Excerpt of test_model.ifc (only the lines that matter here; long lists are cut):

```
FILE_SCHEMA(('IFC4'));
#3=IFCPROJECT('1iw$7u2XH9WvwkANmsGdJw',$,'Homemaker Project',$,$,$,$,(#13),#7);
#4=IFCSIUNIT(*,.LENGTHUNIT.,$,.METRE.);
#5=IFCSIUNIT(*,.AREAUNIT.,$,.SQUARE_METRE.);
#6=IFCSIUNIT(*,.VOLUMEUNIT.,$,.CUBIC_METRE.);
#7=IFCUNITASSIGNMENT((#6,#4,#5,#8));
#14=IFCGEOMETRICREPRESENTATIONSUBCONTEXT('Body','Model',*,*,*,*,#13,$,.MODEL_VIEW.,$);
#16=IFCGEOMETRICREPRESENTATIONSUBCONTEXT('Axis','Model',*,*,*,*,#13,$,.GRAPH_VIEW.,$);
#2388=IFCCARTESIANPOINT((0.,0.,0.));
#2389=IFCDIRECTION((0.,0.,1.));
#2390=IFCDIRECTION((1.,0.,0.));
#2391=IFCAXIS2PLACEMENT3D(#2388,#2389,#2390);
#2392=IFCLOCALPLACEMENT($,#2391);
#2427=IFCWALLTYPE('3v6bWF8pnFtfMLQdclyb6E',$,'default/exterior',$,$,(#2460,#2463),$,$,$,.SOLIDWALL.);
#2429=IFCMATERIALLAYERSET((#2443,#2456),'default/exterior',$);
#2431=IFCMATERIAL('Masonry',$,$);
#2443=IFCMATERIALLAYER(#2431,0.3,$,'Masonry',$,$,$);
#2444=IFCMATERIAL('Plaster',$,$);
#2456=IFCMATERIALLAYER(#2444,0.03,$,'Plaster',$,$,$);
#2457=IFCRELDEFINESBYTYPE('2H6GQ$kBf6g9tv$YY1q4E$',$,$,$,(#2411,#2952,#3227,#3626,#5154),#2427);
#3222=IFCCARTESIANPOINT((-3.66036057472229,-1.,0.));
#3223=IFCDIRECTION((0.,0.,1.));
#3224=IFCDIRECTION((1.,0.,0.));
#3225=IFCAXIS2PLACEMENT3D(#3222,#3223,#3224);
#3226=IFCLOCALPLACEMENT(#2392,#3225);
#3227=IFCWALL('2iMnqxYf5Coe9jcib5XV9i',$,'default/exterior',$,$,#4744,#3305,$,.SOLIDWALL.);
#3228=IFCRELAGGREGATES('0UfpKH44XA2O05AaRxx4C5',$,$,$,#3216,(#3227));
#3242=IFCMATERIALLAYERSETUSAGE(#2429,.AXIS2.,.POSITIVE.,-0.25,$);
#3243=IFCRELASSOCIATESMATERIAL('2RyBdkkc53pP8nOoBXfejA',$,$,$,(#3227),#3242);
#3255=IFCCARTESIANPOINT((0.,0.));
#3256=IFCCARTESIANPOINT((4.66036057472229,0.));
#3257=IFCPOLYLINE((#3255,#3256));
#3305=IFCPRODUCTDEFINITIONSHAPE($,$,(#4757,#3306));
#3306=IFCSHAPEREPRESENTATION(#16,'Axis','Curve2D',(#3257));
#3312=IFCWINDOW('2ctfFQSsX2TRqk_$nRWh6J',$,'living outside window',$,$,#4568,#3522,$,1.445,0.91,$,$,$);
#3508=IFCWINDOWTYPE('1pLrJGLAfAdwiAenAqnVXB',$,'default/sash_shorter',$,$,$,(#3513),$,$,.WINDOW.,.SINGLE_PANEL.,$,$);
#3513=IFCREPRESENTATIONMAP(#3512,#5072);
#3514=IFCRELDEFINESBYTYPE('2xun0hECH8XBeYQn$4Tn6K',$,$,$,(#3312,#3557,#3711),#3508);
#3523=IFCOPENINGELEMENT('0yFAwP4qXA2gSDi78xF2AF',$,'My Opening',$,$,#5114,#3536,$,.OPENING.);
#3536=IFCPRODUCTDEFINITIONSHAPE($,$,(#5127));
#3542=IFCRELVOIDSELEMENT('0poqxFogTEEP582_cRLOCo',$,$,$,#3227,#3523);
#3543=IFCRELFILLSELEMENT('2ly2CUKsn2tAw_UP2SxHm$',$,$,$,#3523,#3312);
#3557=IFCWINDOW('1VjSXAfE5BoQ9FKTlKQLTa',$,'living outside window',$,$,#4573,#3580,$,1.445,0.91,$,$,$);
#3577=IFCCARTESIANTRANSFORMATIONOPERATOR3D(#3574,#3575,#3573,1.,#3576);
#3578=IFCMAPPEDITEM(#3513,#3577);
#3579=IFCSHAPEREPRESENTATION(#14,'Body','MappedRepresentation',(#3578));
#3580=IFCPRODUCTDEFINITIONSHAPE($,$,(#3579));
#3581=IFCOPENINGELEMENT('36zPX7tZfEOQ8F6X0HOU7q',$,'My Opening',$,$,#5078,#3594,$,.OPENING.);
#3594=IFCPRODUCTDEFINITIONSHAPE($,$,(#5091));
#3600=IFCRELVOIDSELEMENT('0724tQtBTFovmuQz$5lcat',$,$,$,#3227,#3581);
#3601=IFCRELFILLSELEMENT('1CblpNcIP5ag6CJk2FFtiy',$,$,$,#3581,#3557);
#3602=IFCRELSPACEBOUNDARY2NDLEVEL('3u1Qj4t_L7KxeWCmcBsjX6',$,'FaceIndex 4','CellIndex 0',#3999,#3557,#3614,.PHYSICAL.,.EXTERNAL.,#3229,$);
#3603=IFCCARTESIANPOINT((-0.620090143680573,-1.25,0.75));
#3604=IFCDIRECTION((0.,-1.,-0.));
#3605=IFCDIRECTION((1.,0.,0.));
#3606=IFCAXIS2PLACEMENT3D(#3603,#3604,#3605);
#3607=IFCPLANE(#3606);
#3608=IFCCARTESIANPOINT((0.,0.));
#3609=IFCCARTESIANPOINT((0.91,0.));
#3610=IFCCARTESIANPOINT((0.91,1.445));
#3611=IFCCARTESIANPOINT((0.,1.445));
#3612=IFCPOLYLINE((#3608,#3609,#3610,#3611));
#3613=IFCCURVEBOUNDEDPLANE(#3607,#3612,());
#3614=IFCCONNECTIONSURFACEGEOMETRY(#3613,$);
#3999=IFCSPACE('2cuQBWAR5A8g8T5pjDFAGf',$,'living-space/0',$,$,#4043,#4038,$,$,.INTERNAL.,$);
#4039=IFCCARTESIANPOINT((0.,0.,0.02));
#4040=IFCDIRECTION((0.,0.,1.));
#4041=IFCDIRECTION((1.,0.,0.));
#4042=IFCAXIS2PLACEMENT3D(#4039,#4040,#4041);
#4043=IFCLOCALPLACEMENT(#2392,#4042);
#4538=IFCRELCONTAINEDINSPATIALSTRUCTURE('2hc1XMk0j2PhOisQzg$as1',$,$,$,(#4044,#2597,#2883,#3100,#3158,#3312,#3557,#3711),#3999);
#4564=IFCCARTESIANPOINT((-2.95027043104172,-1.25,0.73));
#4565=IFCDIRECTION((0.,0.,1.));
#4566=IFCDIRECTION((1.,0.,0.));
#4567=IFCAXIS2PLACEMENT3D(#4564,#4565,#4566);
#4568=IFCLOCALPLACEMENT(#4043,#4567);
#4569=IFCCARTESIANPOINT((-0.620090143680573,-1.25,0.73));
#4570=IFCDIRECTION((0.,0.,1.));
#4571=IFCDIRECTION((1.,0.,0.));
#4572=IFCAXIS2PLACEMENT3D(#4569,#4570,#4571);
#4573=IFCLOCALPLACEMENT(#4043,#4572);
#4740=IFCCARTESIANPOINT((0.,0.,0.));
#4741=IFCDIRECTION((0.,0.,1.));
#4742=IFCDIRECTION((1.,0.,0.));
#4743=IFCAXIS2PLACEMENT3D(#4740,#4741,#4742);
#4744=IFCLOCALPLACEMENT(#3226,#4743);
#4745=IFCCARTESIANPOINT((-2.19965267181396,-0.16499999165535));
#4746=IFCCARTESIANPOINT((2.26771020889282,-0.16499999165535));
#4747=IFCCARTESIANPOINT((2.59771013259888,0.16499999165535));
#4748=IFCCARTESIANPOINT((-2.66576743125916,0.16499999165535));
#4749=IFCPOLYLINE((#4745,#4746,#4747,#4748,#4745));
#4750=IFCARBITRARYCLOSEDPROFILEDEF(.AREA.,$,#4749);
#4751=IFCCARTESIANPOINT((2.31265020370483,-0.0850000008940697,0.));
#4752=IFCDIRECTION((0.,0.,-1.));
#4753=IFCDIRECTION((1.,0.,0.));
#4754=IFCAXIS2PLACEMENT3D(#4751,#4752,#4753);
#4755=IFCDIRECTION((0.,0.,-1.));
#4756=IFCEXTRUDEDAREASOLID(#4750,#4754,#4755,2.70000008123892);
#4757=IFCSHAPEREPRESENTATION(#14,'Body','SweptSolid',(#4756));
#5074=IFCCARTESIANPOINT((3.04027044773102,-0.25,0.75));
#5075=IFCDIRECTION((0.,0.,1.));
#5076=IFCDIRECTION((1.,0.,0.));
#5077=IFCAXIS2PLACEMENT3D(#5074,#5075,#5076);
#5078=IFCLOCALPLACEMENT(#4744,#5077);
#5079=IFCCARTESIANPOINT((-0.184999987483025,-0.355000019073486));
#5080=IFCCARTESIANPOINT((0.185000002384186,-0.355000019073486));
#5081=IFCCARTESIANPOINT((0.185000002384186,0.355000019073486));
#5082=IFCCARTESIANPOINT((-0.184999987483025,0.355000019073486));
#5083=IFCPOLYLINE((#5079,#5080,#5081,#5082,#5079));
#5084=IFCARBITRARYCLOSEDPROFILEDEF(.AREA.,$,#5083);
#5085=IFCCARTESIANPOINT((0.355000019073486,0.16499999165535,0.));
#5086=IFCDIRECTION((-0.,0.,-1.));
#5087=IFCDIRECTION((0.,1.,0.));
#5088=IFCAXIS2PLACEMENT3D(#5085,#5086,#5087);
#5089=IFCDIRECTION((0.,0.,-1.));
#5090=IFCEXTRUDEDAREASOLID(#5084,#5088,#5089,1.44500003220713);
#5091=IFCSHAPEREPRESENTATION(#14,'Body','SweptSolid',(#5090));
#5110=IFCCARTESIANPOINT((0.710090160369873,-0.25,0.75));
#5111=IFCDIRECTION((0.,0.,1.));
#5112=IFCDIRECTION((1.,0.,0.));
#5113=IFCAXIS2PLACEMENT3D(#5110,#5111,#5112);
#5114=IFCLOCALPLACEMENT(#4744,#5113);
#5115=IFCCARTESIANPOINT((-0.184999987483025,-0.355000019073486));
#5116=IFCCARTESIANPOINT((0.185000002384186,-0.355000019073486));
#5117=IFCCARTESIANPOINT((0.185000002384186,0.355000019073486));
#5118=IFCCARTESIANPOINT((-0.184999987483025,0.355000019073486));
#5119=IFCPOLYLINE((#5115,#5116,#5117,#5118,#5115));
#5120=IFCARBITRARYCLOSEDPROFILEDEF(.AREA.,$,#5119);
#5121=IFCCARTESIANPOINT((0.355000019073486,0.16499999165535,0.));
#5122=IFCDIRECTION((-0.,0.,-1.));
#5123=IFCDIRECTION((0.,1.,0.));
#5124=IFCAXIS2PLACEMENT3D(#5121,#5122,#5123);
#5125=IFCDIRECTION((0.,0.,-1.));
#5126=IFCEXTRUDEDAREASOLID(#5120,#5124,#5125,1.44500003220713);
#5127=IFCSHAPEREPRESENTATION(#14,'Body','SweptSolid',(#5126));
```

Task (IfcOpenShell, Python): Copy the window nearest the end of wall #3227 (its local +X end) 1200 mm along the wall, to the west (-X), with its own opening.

```python
import numpy as np
import ifcopenshell
import ifcopenshell.api.feature
import ifcopenshell.api.geometry
import ifcopenshell.api.root
import ifcopenshell.geom
import ifcopenshell.util.element
import ifcopenshell.util.placement
import ifcopenshell.util.shape
import ifcopenshell.util.unit

model = ifcopenshell.open("test_model.ifc")
unit_scale = ifcopenshell.util.unit.calculate_unit_scale(model)
settings = ifcopenshell.geom.settings()


def volume(element):
    """Net volume in cubic metres, openings subtracted."""
    shape = ifcopenshell.geom.create_shape(settings, element)
    return ifcopenshell.util.shape.get_volume(shape.geometry)


window = model.by_guid("1VjSXAfE5BoQ9FKTlKQLTa")
opening = window.FillsVoids[0].RelatingOpeningElement
wall = opening.VoidsElements[0].RelatingBuildingElement
before = volume(wall)
shift = ifcopenshell.util.placement.get_local_placement(wall.ObjectPlacement)[:3, 0] * -1.2 / unit_scale

# copy_class copies the void relationship, type, container and properties, but no geometry.
new_opening = ifcopenshell.api.root.copy_class(model, product=opening)
new_opening.Representation = ifcopenshell.util.element.copy_deep(
    model, opening.Representation, exclude=["IfcGeometricRepresentationContext", "IfcRepresentationMap"]
)
new_window = ifcopenshell.api.root.copy_class(model, product=window)
new_window.Representation = ifcopenshell.util.element.copy_deep(
    model, window.Representation, exclude=["IfcGeometricRepresentationContext", "IfcRepresentationMap"]
)
ifcopenshell.api.feature.add_filling(model, opening=new_opening, element=new_window)

for old, new in ((opening, new_opening), (window, new_window)):
    matrix = ifcopenshell.util.placement.get_local_placement(old.ObjectPlacement)
    matrix[:3, 3] += shift
    ifcopenshell.api.geometry.edit_object_placement(model, product=new, matrix=matrix, is_si=False)

# The copied space boundaries still share their surfaces with the original.
for rel in new_window.ProvidesBoundaries:
    if rel.ConnectionGeometry:
        rel.ConnectionGeometry = ifcopenshell.util.element.copy_deep(model, rel.ConnectionGeometry)

# Space boundary surfaces are stored in each space's coordinates; move them too.
for rel in new_window.ProvidesBoundaries:
    if not rel.ConnectionGeometry:
        continue
    surface = rel.ConnectionGeometry.SurfaceOnRelatingElement.BasisSurface
    space_matrix = ifcopenshell.util.placement.get_local_placement(rel.RelatingSpace.ObjectPlacement)
    point = np.array(surface.Position.Location.Coordinates) + space_matrix[:3, :3].T @ shift
    surface.Position = model.createIfcAxis2Placement3D(
        model.createIfcCartesianPoint(point.tolist()), surface.Position.Axis, surface.Position.RefDirection
    )

after = volume(wall)

print(f"wall volume {before:.3f} -> {after:.3f} m3")

model.write("test_model_v2.ifc")
```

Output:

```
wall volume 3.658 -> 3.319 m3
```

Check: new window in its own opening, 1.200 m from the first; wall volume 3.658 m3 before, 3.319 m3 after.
